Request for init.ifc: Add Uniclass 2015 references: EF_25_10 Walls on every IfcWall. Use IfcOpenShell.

First a look at what the model holds.

```python
import ifcopenshell

model = ifcopenshell.open("init.ifc")
print(model.schema)
print("classifications:", [c.Name for c in model.by_type("IfcClassification")])
for ifc_class in ("IfcDoor", "IfcRoof", "IfcStair", "IfcWall", "IfcWindow"):
    print(ifc_class, len(model.by_type(ifc_class)))
```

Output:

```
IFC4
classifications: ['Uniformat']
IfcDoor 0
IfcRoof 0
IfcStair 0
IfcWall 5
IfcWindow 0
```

```python
import ifcopenshell
import ifcopenshell.api.classification

model = ifcopenshell.open("init.ifc")

system = ifcopenshell.api.classification.add_classification(model, classification="Uniclass 2015")

codes = {
    "IfcWall": ("EF_25_10", "Walls"),
}
for ifc_class, (code, name) in codes.items():
    products = model.by_type(ifc_class)
    ifcopenshell.api.classification.add_reference(
        model, products=products, classification=system, identification=code, name=name
    )
    print(code, len(products))

model.write("init-out.ifc")
```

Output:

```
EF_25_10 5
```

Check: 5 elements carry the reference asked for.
